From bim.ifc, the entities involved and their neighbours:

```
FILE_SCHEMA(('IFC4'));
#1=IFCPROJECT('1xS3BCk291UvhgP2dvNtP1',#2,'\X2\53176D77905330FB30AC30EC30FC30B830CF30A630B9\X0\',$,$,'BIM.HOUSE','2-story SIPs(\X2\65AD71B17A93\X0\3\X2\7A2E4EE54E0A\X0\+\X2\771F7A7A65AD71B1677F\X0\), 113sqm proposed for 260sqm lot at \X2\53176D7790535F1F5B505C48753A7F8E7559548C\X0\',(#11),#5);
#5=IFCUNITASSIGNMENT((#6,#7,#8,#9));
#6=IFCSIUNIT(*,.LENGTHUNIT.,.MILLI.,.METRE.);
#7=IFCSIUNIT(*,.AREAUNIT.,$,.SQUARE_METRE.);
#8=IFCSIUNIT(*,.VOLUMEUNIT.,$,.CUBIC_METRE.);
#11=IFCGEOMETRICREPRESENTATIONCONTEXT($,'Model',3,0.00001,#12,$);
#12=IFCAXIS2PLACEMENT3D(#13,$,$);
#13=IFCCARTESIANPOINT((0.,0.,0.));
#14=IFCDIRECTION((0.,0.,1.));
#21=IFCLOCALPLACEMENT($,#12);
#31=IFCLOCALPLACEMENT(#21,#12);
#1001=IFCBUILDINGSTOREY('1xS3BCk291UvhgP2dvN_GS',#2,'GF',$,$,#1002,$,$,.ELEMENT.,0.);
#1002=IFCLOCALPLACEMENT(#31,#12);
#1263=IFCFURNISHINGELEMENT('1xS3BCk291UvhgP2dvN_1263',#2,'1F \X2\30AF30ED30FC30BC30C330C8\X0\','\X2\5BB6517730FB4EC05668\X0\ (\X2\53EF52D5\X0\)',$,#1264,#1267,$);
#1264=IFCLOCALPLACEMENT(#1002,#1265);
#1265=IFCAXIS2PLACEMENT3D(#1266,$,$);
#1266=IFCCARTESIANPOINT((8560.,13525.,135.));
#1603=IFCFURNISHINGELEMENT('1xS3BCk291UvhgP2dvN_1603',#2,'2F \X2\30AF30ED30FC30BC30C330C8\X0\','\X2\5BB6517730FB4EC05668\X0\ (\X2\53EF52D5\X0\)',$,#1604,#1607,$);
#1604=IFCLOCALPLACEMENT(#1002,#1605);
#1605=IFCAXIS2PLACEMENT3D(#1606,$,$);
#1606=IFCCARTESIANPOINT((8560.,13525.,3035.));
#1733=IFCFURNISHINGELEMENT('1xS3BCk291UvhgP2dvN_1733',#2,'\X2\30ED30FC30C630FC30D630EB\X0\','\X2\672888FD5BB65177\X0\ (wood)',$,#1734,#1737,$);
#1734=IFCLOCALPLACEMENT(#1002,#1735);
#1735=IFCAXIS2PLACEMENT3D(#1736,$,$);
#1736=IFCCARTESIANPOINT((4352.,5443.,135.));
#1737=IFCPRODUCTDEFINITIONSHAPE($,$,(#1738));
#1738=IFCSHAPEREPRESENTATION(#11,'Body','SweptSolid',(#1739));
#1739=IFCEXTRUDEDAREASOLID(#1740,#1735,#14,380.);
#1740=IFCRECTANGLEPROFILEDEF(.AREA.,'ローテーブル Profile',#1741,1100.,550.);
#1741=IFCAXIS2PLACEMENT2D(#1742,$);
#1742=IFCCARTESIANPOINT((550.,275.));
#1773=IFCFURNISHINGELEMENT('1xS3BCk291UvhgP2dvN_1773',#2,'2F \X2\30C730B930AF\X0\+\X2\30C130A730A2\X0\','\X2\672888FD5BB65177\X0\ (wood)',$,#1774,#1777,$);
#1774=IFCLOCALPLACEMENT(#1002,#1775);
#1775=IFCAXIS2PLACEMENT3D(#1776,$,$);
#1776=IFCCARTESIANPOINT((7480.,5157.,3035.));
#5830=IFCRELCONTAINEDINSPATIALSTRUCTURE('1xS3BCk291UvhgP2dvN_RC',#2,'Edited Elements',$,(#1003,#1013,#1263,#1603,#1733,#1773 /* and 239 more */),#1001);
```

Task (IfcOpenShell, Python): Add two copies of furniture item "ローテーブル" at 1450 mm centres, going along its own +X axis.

```python
import ifcopenshell
import ifcopenshell.api.geometry
import ifcopenshell.api.root
import ifcopenshell.util.element
import ifcopenshell.util.placement
import ifcopenshell.util.unit

model = ifcopenshell.open("bim.ifc")
unit_scale = ifcopenshell.util.unit.calculate_unit_scale(model)


def reuse_history(source, copy):
    """copy_class also copies each property set's owner history, people and application; keep the originals."""
    for rel in copy.IsDefinedBy:
        if rel.is_a("IfcRelDefinesByProperties") and (history := rel.RelatingPropertyDefinition.OwnerHistory):
            rel.RelatingPropertyDefinition.OwnerHistory = source.OwnerHistory
            ifcopenshell.util.element.remove_deep2(model, history)


source = model.by_guid("1xS3BCk291UvhgP2dvN_1733")
base = ifcopenshell.util.placement.get_local_placement(source.ObjectPlacement)
step = base[:3, 0] * 1.45 / unit_scale

for i in range(1, 3):
    copy = ifcopenshell.api.root.copy_class(model, product=source)
    copy.Representation = ifcopenshell.util.element.copy_deep(
        model, source.Representation, exclude=["IfcGeometricRepresentationContext", "IfcRepresentationMap"]
    )
    reuse_history(source, copy)
    matrix = base.copy()
    matrix[:3, 3] += i * step
    print("added at", matrix[:3, 3].round(3) + 0.0)
    ifcopenshell.api.geometry.edit_object_placement(model, product=copy, matrix=matrix, is_si=False)

model.write("bim_updated.ifc")
```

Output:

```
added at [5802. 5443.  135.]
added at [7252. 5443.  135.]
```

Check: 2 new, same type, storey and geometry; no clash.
